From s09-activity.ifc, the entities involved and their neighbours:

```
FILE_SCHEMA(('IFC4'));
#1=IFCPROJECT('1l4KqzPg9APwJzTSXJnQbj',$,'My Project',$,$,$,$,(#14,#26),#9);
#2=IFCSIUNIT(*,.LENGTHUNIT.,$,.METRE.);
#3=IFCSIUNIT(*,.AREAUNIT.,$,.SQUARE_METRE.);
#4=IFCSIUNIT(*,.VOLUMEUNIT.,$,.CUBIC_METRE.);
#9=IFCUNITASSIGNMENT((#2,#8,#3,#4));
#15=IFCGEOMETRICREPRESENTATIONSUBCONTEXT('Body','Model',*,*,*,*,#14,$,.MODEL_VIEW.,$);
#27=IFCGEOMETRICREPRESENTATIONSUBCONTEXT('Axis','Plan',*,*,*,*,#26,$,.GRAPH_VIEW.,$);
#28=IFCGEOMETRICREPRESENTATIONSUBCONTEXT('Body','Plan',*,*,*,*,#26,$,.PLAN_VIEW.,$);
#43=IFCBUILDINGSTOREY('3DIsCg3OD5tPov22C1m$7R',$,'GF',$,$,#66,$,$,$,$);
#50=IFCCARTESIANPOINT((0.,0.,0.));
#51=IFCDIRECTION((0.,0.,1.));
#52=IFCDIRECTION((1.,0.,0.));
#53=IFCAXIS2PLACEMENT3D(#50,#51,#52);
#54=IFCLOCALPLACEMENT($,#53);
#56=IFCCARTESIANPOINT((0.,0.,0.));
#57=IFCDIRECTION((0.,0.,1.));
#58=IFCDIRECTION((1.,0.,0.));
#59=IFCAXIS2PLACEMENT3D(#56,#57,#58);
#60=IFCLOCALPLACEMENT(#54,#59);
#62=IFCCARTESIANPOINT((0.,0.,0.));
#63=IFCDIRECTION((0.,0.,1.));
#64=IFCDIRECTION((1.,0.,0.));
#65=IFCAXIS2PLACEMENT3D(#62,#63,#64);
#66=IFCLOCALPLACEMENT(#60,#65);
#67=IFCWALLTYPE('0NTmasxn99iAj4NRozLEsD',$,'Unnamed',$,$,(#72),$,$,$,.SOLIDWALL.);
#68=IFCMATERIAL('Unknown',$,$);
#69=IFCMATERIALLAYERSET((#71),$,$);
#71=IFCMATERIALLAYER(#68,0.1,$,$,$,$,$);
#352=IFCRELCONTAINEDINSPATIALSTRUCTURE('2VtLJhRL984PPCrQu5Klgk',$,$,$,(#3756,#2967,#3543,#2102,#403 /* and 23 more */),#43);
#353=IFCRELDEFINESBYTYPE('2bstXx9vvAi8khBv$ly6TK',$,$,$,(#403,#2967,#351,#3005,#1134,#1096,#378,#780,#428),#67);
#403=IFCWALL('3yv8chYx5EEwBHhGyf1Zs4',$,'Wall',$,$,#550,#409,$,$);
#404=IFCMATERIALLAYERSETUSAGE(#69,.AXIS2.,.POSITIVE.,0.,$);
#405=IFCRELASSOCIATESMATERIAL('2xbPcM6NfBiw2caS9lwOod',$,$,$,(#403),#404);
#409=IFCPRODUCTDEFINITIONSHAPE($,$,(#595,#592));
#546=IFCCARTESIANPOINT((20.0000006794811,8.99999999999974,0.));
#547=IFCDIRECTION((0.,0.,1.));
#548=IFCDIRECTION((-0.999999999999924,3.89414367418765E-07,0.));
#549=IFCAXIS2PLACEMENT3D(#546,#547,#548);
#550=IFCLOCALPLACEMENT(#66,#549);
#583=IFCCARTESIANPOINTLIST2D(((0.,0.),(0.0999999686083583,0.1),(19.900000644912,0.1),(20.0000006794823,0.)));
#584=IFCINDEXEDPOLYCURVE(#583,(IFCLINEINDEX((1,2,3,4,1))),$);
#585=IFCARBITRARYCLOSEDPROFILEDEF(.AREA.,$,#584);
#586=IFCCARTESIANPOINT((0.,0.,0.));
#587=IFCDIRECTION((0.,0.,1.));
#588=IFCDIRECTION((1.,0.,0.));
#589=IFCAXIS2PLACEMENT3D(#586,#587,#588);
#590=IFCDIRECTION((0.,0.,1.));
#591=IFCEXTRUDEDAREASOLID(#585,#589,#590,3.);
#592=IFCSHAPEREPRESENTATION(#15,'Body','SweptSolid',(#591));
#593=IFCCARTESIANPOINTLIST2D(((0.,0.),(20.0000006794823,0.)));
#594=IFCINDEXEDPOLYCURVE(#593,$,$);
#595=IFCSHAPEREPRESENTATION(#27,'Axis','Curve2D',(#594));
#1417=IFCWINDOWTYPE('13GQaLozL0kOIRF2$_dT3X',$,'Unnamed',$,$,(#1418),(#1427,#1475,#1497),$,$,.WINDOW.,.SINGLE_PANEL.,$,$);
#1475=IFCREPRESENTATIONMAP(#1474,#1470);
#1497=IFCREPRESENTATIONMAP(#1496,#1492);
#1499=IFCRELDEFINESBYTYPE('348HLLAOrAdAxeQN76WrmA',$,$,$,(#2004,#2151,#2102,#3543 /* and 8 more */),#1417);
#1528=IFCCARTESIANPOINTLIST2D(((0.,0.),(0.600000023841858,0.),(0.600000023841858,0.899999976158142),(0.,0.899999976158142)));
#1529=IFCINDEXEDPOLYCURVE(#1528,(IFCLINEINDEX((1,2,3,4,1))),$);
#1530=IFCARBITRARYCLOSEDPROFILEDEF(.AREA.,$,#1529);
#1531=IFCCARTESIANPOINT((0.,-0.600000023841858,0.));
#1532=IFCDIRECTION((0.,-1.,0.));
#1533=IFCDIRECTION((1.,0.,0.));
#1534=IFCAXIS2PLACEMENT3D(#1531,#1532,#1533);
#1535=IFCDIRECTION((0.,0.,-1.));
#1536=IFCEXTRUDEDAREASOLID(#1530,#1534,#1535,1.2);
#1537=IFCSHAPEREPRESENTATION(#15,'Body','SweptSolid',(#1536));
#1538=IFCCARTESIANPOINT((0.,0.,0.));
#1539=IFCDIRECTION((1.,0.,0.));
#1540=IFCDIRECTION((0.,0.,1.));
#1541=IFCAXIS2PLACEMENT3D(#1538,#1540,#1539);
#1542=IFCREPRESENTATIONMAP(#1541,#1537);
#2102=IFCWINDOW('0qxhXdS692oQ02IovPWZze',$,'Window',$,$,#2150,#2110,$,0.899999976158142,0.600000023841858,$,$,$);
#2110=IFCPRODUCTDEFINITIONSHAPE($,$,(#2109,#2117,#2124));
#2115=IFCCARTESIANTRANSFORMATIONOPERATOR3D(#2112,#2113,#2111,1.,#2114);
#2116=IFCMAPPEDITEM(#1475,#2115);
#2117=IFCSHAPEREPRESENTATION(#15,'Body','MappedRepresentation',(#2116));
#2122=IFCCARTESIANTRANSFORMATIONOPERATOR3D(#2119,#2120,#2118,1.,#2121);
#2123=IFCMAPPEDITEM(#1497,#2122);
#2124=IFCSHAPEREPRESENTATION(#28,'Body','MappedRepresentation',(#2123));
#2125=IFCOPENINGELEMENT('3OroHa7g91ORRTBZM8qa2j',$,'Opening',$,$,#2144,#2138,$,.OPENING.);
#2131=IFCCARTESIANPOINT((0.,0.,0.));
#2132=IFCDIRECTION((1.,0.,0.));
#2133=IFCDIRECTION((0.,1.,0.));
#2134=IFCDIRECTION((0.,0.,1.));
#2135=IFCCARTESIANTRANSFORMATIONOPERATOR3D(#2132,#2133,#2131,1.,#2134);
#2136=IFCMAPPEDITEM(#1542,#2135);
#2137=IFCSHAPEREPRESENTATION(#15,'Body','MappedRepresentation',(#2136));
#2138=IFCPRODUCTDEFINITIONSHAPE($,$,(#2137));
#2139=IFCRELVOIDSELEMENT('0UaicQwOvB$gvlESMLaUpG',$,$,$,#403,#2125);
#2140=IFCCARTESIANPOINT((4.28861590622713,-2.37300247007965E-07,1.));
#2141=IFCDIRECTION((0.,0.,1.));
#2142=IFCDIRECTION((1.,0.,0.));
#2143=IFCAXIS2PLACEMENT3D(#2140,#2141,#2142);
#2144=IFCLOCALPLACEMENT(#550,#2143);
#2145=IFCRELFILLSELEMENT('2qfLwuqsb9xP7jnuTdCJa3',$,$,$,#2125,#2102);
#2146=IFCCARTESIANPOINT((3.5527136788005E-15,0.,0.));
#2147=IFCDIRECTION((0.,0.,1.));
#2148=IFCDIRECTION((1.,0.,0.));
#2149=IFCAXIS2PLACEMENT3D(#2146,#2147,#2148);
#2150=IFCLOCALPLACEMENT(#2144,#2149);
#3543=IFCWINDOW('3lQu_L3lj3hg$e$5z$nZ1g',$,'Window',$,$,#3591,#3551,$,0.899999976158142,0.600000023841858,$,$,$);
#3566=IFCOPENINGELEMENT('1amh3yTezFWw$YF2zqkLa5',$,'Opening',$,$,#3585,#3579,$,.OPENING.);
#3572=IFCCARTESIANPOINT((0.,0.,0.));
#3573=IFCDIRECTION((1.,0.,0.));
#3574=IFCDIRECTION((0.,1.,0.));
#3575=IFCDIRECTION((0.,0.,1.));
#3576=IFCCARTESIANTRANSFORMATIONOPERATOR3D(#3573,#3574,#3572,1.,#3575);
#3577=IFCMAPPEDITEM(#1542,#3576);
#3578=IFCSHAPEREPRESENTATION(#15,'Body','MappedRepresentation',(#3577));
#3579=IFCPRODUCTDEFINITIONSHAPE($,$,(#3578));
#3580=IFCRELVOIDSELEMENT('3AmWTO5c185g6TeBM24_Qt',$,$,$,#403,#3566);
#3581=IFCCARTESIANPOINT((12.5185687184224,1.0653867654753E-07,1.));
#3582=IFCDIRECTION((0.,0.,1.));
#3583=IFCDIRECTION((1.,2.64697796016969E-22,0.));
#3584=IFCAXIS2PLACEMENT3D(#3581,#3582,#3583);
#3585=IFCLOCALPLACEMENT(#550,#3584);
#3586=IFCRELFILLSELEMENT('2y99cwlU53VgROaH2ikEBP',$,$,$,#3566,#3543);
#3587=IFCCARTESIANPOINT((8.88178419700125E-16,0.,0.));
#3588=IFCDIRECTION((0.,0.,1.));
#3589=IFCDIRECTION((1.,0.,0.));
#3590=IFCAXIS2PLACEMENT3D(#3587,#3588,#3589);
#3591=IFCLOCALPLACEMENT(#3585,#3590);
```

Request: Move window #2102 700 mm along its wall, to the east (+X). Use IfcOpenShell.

```python
import ifcopenshell
import ifcopenshell.api.geometry
import ifcopenshell.util.placement

model = ifcopenshell.open("s09-activity.ifc")

window = model.by_guid("0qxhXdS692oQ02IovPWZze")
opening = window.FillsVoids[0].RelatingOpeningElement
wall = opening.VoidsElements[0].RelatingBuildingElement

wall_matrix = ifcopenshell.util.placement.get_local_placement(wall.ObjectPlacement)
shift = wall_matrix[:3, 0] * -0.7
before = ifcopenshell.util.placement.get_local_placement(window.ObjectPlacement)[:3, 3].copy()

# The window is placed relative to its opening, so it follows when the opening moves.
matrix = ifcopenshell.util.placement.get_local_placement(opening.ObjectPlacement)
matrix[:3, 3] += shift
ifcopenshell.api.geometry.edit_object_placement(
    model, product=opening, matrix=matrix, is_si=False, should_transform_children=True
)

after = ifcopenshell.util.placement.get_local_placement(window.ObjectPlacement)[:3, 3]
print("window moved by", (after - before).round(3) + 0.0)

model.write("s09-activity-out.ifc")
```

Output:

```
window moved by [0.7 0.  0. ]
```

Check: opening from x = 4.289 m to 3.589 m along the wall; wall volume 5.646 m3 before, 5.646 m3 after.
